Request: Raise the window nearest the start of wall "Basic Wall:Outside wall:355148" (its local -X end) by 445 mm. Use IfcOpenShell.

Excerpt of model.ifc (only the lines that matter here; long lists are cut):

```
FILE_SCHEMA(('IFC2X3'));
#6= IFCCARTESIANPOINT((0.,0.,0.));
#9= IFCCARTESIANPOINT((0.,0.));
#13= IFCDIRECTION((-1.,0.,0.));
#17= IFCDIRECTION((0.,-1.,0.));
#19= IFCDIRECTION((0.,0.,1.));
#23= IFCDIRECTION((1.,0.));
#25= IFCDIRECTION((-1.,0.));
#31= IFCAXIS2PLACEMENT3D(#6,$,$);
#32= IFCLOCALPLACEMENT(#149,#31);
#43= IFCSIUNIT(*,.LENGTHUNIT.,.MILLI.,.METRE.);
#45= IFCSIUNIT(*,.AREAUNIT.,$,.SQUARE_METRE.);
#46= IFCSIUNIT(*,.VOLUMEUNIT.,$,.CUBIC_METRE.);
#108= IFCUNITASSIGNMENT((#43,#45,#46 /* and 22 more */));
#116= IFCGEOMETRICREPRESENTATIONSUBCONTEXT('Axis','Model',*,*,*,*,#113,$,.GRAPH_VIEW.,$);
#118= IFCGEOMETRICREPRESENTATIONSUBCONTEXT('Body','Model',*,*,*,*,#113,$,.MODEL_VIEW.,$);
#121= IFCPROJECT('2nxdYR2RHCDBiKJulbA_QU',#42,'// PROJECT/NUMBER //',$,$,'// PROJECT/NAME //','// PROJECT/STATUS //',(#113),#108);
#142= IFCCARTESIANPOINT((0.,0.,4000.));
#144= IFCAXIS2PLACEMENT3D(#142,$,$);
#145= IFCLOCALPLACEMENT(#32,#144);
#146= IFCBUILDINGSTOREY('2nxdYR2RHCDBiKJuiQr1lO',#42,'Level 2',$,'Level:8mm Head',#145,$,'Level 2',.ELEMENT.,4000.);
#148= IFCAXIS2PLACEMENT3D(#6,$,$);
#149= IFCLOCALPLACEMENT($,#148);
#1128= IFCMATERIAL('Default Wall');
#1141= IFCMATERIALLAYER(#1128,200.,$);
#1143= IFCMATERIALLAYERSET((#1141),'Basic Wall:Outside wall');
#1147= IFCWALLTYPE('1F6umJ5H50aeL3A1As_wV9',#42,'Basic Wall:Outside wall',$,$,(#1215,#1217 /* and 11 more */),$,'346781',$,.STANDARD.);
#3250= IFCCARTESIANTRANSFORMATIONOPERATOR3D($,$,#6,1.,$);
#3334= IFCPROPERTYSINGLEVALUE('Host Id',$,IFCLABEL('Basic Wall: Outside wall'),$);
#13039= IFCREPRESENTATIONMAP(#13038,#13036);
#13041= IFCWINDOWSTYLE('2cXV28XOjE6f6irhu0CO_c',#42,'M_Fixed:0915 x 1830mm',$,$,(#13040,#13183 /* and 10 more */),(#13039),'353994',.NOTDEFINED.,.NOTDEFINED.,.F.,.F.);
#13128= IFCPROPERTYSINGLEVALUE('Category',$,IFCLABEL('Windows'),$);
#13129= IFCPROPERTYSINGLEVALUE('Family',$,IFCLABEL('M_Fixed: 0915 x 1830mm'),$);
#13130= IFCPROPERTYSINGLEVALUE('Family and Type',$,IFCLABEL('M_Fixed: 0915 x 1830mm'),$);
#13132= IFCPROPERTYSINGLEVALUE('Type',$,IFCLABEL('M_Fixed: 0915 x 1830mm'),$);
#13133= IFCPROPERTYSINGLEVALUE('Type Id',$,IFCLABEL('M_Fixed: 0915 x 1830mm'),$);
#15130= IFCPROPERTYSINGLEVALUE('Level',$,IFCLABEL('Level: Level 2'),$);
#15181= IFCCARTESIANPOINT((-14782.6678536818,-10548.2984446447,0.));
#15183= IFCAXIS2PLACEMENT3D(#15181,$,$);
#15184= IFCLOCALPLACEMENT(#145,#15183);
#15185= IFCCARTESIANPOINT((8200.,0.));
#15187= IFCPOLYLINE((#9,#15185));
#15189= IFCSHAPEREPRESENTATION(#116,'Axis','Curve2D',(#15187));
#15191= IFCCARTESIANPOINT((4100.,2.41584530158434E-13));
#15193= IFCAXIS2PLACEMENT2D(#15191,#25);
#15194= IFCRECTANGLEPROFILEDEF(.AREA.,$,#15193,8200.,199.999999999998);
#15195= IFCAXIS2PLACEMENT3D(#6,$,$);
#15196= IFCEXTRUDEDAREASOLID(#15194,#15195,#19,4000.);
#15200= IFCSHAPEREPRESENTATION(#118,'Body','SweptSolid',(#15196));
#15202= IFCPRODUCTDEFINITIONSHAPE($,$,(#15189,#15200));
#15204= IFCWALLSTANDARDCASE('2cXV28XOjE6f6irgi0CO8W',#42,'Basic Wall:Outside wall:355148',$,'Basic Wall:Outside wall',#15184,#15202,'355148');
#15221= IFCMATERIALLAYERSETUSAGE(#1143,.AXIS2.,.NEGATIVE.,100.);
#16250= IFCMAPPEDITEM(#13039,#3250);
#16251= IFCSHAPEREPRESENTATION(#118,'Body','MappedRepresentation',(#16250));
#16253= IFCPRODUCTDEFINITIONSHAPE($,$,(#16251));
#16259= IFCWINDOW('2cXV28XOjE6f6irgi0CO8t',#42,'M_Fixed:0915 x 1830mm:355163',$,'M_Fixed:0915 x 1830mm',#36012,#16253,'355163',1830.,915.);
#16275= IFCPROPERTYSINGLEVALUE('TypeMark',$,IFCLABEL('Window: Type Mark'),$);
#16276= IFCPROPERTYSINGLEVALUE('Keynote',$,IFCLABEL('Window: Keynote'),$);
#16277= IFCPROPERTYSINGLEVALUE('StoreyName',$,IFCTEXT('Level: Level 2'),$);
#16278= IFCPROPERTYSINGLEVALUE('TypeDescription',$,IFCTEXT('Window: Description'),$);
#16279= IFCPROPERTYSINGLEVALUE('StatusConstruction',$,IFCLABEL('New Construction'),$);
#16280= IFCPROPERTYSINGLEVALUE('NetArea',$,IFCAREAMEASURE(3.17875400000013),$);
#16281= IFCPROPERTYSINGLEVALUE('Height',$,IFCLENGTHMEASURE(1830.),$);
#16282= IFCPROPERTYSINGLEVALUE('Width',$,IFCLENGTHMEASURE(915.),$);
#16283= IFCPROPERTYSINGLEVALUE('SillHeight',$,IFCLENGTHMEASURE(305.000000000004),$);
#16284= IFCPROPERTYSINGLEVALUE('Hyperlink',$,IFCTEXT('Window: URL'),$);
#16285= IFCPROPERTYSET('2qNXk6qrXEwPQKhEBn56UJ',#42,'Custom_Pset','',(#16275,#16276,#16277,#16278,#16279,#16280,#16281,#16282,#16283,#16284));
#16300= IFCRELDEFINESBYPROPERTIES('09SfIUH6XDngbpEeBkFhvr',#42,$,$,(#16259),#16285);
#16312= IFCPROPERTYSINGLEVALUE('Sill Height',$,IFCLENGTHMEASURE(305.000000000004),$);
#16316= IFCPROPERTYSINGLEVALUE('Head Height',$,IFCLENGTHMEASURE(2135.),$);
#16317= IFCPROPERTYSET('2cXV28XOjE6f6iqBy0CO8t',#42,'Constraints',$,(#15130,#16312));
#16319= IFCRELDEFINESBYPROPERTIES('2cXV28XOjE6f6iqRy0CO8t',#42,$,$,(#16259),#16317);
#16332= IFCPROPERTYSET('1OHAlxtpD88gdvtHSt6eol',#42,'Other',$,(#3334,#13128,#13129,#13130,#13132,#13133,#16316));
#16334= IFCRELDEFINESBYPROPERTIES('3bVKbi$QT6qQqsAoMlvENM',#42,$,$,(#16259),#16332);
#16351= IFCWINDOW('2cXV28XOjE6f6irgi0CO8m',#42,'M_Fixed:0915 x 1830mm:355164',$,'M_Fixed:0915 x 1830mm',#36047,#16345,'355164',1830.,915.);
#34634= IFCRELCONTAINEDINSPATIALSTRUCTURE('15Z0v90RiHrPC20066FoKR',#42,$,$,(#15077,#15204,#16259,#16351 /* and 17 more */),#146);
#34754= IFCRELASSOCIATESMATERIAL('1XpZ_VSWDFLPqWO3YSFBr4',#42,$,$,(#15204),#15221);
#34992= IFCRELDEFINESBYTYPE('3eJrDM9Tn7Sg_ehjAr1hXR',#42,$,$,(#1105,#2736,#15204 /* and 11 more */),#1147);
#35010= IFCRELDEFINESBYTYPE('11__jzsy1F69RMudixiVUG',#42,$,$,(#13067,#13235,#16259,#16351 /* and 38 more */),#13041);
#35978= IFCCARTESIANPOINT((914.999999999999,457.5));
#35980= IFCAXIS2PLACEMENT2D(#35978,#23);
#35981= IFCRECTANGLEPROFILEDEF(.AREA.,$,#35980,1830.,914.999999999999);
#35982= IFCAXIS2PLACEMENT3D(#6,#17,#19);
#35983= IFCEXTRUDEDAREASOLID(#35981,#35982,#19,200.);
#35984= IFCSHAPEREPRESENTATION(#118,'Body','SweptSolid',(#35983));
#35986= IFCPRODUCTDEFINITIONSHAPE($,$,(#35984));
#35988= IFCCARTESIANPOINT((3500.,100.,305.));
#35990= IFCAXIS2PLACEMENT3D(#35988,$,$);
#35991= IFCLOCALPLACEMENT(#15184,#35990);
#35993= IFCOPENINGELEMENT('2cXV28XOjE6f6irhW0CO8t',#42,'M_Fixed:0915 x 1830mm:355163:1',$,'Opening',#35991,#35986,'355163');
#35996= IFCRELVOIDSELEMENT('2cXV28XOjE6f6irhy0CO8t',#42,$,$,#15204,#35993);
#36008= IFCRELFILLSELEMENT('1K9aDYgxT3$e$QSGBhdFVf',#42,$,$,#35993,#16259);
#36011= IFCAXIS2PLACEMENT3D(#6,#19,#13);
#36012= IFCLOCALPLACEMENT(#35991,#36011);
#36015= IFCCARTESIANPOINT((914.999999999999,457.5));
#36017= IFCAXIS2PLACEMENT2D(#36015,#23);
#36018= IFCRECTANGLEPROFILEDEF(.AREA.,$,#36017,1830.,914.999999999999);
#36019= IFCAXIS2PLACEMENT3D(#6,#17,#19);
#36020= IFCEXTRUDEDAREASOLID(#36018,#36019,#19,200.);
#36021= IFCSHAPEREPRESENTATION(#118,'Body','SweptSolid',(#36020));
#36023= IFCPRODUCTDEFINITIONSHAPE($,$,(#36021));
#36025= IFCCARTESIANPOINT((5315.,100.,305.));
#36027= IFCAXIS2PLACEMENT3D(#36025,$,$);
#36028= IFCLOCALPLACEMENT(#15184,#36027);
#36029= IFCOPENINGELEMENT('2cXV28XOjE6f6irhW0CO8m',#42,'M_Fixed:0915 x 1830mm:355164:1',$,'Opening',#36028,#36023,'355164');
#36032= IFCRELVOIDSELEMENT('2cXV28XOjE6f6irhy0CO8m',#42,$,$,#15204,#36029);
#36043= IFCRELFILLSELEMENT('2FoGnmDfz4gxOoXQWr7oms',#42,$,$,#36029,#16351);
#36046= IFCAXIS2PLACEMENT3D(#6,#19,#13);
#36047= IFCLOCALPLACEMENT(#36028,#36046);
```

```python
import numpy as np
import ifcopenshell
import ifcopenshell.api.geometry
import ifcopenshell.api.pset
import ifcopenshell.util.element
import ifcopenshell.util.placement
import ifcopenshell.util.unit

model = ifcopenshell.open("model.ifc")
unit_scale = ifcopenshell.util.unit.calculate_unit_scale(model)

window = model.by_id(16259)
opening = window.FillsVoids[0].RelatingOpeningElement
dz = 445.0

shift = np.array([0.0, 0.0, dz])
# The window is placed relative to its opening, so it follows when the opening moves.
matrix = ifcopenshell.util.placement.get_local_placement(opening.ObjectPlacement)
matrix[:3, 3] += shift
ifcopenshell.api.geometry.edit_object_placement(
    model, product=opening, matrix=matrix, is_si=False, should_transform_children=True
)

# Keep the stored heights in step.
pset = model.by_id(ifcopenshell.util.element.get_pset(window, "Custom_Pset", should_inherit=False)["id"])
ifcopenshell.api.pset.edit_pset(model, pset=pset, properties={
    "SillHeight": model.create_entity("IfcLengthMeasure", ifcopenshell.util.element.get_pset(window, "Constraints", "Sill Height") + dz),
})
pset = model.by_id(ifcopenshell.util.element.get_pset(window, "Constraints", should_inherit=False)["id"])
ifcopenshell.api.pset.edit_pset(model, pset=pset, properties={
    "Sill Height": model.create_entity("IfcLengthMeasure", ifcopenshell.util.element.get_pset(window, "Constraints", "Sill Height") + dz),
})
pset = model.by_id(ifcopenshell.util.element.get_pset(window, "Other", should_inherit=False)["id"])
ifcopenshell.api.pset.edit_pset(model, pset=pset, properties={
    "Head Height": model.create_entity("IfcLengthMeasure", ifcopenshell.util.element.get_pset(window, "Other", "Head Height") + dz),
})

print(f"moved by {dz * unit_scale:+.3f} m")

model.write("model_rev.ifc")
```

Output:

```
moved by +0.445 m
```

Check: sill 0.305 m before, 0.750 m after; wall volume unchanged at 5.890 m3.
